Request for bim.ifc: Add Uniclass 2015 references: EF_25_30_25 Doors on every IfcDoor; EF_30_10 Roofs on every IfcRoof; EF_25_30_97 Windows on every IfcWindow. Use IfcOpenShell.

First a look at what the model holds.

```python
import ifcopenshell

model = ifcopenshell.open("bim.ifc")
print(model.schema)
print("classifications:", [c.Name for c in model.by_type("IfcClassification")])
for ifc_class in ("IfcDoor", "IfcRoof", "IfcStair", "IfcWall", "IfcWindow"):
    print(ifc_class, len(model.by_type(ifc_class)))
```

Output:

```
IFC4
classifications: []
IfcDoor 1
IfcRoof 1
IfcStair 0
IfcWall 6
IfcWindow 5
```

```python
import ifcopenshell
import ifcopenshell.api.classification

model = ifcopenshell.open("bim.ifc")

system = ifcopenshell.api.classification.add_classification(model, classification="Uniclass 2015")

codes = {
    "IfcDoor": ("EF_25_30_25", "Doors"),
    "IfcRoof": ("EF_30_10", "Roofs"),
    "IfcWindow": ("EF_25_30_97", "Windows"),
}
for ifc_class, (code, name) in codes.items():
    products = model.by_type(ifc_class)
    ifcopenshell.api.classification.add_reference(
        model, products=products, classification=system, identification=code, name=name
    )
    print(code, len(products))

model.write("bim_rev.ifc")
```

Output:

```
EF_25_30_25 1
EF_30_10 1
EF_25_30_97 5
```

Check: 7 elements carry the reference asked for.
